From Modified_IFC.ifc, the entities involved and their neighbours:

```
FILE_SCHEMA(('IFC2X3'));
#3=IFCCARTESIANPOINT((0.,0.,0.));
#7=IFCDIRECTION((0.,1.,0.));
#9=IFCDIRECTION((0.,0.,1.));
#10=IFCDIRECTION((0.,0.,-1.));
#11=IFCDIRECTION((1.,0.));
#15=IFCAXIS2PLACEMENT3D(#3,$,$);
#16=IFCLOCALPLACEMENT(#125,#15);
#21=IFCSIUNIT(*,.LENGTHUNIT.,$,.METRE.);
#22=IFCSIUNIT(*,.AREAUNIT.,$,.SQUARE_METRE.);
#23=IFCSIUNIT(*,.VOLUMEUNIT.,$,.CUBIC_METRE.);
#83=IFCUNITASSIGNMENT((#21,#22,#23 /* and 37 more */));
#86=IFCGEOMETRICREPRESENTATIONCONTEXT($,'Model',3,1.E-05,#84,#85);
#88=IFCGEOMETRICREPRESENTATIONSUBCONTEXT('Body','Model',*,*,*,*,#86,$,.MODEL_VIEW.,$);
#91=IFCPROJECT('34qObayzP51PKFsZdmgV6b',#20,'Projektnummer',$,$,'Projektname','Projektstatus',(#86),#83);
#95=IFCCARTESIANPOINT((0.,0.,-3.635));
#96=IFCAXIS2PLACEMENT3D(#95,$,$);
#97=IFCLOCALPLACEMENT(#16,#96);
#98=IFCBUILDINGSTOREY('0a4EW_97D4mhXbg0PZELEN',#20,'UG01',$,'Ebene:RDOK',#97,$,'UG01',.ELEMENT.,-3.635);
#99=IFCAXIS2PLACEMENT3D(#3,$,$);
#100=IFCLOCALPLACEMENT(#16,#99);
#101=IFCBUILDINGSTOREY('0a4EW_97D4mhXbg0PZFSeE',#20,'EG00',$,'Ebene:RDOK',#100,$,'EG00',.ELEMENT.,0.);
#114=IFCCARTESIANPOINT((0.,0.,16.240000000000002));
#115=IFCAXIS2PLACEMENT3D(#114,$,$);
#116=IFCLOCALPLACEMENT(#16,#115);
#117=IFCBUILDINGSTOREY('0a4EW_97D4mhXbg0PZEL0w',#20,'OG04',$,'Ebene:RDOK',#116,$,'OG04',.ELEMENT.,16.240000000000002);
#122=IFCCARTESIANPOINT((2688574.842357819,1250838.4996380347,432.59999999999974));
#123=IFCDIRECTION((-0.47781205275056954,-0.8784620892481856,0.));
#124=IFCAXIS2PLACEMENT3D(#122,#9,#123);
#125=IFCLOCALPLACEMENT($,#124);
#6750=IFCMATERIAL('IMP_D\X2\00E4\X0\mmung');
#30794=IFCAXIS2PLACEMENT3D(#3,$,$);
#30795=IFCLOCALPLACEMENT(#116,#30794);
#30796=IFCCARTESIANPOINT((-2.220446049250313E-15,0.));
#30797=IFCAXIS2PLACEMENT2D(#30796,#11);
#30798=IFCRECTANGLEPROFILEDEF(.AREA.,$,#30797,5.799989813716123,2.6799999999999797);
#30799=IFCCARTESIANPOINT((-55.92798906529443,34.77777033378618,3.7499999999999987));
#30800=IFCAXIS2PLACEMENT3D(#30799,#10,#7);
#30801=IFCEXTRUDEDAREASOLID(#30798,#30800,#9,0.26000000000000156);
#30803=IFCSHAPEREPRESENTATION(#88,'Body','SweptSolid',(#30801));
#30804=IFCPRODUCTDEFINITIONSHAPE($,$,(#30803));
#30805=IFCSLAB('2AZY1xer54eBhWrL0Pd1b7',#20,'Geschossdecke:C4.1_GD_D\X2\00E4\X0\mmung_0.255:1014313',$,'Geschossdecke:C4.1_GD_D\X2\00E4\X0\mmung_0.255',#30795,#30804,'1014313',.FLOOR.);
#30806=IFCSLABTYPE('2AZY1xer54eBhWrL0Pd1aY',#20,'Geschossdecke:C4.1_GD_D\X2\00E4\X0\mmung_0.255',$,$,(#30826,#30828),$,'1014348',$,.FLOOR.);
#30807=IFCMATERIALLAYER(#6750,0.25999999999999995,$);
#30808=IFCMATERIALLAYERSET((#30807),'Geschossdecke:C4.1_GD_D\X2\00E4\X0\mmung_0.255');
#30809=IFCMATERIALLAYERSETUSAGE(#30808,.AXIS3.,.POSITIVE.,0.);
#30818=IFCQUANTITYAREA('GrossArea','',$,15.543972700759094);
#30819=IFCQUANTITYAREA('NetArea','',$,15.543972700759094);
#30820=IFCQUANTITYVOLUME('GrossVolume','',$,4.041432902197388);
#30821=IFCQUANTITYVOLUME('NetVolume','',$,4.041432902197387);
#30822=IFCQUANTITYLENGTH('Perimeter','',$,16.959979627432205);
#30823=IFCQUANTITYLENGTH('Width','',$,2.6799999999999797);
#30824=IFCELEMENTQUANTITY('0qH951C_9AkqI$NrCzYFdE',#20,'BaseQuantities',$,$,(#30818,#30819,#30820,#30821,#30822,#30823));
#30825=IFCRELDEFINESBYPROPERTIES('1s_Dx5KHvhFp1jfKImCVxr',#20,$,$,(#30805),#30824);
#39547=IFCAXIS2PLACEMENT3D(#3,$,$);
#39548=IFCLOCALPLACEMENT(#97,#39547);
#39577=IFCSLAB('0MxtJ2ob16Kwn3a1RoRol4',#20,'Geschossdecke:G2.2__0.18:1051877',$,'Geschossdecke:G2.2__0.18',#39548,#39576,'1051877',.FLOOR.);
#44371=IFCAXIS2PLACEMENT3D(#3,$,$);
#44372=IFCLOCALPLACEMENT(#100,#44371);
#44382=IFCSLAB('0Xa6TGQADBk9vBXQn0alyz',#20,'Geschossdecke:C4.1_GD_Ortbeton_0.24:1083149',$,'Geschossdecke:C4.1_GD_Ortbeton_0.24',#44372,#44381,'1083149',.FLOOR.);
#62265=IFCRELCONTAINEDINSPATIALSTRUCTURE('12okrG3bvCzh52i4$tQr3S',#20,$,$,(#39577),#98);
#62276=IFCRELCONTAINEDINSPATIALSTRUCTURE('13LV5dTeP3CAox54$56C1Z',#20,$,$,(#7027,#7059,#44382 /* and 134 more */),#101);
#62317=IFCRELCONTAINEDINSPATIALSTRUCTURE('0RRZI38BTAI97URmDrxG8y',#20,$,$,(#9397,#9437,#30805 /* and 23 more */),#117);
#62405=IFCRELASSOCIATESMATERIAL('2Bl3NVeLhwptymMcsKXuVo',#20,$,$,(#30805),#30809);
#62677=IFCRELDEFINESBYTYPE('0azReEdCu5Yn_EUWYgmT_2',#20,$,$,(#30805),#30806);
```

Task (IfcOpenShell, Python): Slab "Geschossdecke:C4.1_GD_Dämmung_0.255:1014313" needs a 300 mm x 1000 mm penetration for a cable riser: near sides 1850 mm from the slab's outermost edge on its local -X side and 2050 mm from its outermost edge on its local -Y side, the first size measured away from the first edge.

```python
import numpy as np
import ifcopenshell
import ifcopenshell.api.feature
import ifcopenshell.api.geometry
import ifcopenshell.api.pset
import ifcopenshell.api.root
import ifcopenshell.geom
import ifcopenshell.util.element
import ifcopenshell.util.placement
import ifcopenshell.util.representation
import ifcopenshell.util.shape
import ifcopenshell.util.unit

model = ifcopenshell.open("Modified_IFC.ifc")
unit_scale = ifcopenshell.util.unit.calculate_unit_scale(model)
area_scale = ifcopenshell.util.unit.calculate_unit_scale(model, "AREAUNIT")
volume_scale = ifcopenshell.util.unit.calculate_unit_scale(model, "VOLUMEUNIT")
settings = ifcopenshell.geom.settings()


def volume(element):
    """Net volume in cubic metres, openings subtracted."""
    shape = ifcopenshell.geom.create_shape(settings, element)
    return ifcopenshell.util.shape.get_volume(shape.geometry)


slab = model.by_guid("2AZY1xer54eBhWrL0Pd1b7")
before = volume(slab)

# Extent in the slab's own axes, in metres. The edges named are its -X and -Y sides.
slab_shape = ifcopenshell.geom.create_shape(settings, slab)
vertices = ifcopenshell.util.shape.get_vertices(slab_shape.geometry)
x_min, y_min, bottom = vertices.min(axis=0)
top = vertices[:, 2].max()

opening = ifcopenshell.api.root.create_entity(model, ifc_class="IfcOpeningElement", name="Cable riser opening")
context = ifcopenshell.util.representation.get_context(model, "Model", "Body", "MODEL_VIEW")
width, depth = 0.3, 1
outline = [(0.0, 0.0), (width, 0.0), (width, depth), (0.0, depth), (0.0, 0.0)]
# Overshoot both faces by 50 mm so the cut is clean.
shape = ifcopenshell.api.geometry.add_slab_representation(
    model, context=context, depth=top - bottom + 0.1, polyline=outline
)
ifcopenshell.api.geometry.assign_representation(model, product=opening, representation=shape)

matrix = ifcopenshell.util.placement.get_local_placement(slab.ObjectPlacement)
matrix[:, 3] = matrix @ np.append(np.array([x_min + 1.85, y_min + 2.05, bottom - 0.05]) / unit_scale, 1.0)
ifcopenshell.api.geometry.edit_object_placement(model, product=opening, matrix=matrix, is_si=False)
ifcopenshell.api.feature.add_feature(model, feature=opening, element=slab)

after = volume(slab)

# Update the slab's stored quantities.
qto = model.by_id(ifcopenshell.util.element.get_pset(slab, "BaseQuantities", should_inherit=False)["id"])
ifcopenshell.api.pset.edit_qto(model, qto=qto, properties={
    "NetArea": after / (top - bottom) / area_scale,
    "NetVolume": after / volume_scale,
})

print(f"slab volume {before:.3f} -> {after:.3f} m3")

model.write("Modified_IFC_v2.ifc")
```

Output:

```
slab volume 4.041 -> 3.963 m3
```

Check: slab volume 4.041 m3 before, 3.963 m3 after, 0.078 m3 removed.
